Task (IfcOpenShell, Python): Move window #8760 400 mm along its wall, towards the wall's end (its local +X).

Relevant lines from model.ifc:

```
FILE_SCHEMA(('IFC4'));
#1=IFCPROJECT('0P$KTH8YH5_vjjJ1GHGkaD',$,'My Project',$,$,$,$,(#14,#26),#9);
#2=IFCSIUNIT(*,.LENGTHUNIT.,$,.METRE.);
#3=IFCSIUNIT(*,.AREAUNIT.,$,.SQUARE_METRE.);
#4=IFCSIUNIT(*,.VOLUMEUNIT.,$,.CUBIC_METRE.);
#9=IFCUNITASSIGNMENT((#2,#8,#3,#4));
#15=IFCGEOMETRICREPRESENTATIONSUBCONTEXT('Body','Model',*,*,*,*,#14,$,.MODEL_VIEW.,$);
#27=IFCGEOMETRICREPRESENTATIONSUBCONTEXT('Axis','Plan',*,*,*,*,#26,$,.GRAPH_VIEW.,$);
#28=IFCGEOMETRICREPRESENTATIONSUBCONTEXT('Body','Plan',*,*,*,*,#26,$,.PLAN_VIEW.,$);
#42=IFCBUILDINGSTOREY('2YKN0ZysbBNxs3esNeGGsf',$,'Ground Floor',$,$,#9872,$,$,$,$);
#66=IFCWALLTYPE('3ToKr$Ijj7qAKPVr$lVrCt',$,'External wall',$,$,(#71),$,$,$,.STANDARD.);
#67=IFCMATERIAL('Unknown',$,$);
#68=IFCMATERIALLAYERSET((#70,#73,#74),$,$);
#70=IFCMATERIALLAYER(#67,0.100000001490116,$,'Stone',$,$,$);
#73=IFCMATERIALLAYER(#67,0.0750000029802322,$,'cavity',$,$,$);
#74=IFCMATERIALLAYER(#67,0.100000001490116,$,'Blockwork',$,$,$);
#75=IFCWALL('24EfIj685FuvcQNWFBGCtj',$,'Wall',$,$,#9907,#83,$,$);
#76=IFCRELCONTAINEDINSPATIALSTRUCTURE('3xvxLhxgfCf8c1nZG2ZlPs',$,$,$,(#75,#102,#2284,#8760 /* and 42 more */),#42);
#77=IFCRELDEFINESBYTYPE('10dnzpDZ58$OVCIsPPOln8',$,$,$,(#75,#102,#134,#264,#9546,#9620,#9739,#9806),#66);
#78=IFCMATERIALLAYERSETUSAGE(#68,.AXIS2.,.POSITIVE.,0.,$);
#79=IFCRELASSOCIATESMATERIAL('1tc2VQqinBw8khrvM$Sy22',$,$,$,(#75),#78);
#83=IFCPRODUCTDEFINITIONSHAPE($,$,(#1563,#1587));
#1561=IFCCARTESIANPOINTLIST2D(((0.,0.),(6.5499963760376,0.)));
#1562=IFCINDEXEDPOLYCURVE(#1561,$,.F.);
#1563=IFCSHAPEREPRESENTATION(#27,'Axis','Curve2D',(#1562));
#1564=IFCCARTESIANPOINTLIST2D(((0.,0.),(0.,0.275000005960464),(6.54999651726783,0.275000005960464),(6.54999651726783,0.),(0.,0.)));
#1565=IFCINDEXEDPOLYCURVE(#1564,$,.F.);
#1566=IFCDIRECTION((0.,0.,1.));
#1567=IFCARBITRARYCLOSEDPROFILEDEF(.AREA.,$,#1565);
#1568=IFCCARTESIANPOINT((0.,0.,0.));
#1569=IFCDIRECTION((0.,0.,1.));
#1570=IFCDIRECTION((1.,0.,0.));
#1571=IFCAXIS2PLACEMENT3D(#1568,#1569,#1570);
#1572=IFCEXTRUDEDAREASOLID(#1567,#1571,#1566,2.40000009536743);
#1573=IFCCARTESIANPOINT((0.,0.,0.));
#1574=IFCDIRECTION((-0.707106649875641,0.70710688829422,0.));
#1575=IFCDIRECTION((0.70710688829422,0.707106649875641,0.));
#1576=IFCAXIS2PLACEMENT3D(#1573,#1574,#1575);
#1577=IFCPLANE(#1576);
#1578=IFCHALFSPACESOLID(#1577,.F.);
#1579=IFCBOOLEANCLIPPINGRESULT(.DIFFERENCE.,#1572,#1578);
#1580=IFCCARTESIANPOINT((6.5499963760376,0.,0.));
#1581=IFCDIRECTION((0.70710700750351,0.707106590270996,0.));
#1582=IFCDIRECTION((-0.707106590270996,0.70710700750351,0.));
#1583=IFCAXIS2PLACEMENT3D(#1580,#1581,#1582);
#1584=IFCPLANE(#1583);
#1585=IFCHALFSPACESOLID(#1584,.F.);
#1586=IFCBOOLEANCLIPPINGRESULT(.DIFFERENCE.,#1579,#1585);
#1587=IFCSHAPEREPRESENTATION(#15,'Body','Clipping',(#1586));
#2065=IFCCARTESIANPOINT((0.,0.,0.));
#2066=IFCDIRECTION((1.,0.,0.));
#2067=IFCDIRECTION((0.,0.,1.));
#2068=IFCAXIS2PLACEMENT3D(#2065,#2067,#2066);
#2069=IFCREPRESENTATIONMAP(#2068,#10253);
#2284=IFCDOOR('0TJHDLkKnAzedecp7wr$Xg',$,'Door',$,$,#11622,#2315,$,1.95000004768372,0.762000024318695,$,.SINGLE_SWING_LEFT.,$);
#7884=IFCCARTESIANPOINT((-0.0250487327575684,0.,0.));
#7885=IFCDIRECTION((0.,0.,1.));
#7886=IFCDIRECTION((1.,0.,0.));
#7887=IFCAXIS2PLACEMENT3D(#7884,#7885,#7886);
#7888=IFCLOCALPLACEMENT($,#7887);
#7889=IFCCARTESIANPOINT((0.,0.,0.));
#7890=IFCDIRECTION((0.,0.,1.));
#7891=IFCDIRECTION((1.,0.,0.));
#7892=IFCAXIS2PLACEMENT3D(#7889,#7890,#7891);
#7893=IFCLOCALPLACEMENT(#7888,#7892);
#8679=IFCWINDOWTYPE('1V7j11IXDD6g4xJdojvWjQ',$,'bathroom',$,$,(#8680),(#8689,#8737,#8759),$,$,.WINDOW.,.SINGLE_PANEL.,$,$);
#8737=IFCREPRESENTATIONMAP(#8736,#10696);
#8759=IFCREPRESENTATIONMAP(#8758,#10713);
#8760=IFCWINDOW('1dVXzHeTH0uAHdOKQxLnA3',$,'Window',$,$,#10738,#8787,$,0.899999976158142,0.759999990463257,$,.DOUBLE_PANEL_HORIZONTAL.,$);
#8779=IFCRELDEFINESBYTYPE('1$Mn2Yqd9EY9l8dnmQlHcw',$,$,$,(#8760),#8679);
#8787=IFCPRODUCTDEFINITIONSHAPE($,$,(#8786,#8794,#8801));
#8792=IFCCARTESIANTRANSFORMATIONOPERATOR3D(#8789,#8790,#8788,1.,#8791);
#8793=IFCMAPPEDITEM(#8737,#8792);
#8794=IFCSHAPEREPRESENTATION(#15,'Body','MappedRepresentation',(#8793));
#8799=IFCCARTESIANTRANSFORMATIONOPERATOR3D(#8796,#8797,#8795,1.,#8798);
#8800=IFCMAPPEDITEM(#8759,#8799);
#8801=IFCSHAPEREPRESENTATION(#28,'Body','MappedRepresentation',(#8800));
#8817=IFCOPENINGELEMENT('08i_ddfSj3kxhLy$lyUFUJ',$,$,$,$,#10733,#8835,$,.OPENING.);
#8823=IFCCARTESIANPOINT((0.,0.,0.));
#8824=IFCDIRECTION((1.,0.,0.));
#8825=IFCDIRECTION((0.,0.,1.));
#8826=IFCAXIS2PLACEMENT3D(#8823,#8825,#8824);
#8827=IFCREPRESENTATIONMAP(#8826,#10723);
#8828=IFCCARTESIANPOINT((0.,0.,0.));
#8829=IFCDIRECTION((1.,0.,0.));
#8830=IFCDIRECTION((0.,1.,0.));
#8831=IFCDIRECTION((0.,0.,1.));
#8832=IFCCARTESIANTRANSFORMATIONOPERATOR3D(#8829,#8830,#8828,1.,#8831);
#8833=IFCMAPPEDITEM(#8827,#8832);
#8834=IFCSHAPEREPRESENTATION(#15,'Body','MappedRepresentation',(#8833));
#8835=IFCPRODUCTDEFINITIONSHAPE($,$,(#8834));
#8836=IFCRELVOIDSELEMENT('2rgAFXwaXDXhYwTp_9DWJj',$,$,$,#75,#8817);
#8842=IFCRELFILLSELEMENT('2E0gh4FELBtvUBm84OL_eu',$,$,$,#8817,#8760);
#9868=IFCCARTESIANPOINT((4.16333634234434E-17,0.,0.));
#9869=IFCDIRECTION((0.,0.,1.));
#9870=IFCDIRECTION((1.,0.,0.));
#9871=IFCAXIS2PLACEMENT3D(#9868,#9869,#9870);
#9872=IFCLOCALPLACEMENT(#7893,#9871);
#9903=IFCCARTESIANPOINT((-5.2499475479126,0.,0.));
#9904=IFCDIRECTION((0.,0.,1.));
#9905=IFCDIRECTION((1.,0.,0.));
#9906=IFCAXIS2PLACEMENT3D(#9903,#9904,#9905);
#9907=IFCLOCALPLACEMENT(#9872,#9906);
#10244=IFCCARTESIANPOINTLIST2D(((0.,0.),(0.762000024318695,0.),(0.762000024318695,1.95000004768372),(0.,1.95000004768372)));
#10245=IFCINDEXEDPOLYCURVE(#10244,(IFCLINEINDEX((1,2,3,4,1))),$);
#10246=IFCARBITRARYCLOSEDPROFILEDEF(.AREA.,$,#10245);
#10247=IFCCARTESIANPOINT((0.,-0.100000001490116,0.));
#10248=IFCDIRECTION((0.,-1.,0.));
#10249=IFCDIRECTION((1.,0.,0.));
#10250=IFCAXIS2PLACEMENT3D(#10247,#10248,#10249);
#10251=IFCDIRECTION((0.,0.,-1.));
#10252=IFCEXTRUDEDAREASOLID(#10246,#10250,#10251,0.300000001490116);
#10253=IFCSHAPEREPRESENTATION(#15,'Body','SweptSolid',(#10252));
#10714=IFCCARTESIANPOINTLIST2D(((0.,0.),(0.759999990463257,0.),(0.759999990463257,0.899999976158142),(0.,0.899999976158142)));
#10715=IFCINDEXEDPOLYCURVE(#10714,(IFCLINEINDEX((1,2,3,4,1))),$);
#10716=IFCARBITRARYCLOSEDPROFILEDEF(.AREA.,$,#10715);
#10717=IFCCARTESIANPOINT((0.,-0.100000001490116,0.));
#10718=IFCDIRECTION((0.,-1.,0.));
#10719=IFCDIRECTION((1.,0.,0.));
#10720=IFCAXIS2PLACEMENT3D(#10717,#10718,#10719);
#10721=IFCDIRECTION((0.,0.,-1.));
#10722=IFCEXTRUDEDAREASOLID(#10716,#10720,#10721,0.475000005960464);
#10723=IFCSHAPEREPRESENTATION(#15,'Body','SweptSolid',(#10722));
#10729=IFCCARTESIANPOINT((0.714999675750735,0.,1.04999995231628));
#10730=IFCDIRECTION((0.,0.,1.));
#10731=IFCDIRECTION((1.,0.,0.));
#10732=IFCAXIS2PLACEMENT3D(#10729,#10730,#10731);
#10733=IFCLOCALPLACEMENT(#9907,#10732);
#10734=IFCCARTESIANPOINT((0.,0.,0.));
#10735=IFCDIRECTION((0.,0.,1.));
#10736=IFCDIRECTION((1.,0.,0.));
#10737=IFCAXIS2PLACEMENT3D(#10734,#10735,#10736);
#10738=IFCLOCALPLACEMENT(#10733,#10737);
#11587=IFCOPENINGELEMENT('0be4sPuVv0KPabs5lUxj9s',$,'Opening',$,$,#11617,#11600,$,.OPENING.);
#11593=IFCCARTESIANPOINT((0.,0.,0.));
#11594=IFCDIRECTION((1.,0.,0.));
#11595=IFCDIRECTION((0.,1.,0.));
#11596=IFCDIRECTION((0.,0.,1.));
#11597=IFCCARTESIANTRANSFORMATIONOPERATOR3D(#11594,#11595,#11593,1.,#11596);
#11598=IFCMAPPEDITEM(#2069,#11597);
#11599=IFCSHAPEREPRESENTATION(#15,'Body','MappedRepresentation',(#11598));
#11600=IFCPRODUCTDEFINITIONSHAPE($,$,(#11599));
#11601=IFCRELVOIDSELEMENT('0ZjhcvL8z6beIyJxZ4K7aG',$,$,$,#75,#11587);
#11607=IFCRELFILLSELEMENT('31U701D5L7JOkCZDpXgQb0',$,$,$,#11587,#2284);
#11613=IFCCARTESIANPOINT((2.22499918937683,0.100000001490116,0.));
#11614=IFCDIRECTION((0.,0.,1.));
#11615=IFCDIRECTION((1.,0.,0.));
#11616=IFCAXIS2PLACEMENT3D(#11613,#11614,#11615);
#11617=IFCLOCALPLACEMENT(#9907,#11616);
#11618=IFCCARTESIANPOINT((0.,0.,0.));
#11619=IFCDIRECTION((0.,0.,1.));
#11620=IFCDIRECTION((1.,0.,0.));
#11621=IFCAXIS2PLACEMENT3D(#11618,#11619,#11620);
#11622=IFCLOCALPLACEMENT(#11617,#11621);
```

```python
import ifcopenshell
import ifcopenshell.api.geometry
import ifcopenshell.util.placement
import ifcopenshell.util.unit

model = ifcopenshell.open("model.ifc")
unit_scale = ifcopenshell.util.unit.calculate_unit_scale(model)

window = model.by_id(8760)
opening = window.FillsVoids[0].RelatingOpeningElement
wall = opening.VoidsElements[0].RelatingBuildingElement

wall_matrix = ifcopenshell.util.placement.get_local_placement(wall.ObjectPlacement)
shift = wall_matrix[:3, 0] * 0.4 / unit_scale
before = ifcopenshell.util.placement.get_local_placement(window.ObjectPlacement)[:3, 3].copy()

# The window is placed relative to its opening, so it follows when the opening moves.
matrix = ifcopenshell.util.placement.get_local_placement(opening.ObjectPlacement)
matrix[:3, 3] += shift
ifcopenshell.api.geometry.edit_object_placement(
    model, product=opening, matrix=matrix, is_si=False, should_transform_children=True
)

after = ifcopenshell.util.placement.get_local_placement(window.ObjectPlacement)[:3, 3]
print("window moved by", (after - before).round(3) + 0.0)

model.write("model_updated.ifc")
```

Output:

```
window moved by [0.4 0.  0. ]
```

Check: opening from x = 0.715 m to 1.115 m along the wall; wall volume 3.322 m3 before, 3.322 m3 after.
